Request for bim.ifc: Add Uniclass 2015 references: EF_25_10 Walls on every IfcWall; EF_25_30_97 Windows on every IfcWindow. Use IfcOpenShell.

First a look at what the model holds.

```python
import ifcopenshell

model = ifcopenshell.open("bim.ifc")
print(model.schema)
print("classifications:", [c.Name for c in model.by_type("IfcClassification")])
for ifc_class in ("IfcDoor", "IfcRoof", "IfcStair", "IfcWall", "IfcWindow"):
    print(ifc_class, len(model.by_type(ifc_class)))
```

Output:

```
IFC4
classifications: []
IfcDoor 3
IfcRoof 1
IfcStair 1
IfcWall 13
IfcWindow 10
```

```python
import ifcopenshell
import ifcopenshell.api.classification

model = ifcopenshell.open("bim.ifc")

system = ifcopenshell.api.classification.add_classification(model, classification="Uniclass 2015")

codes = {
    "IfcWall": ("EF_25_10", "Walls"),
    "IfcWindow": ("EF_25_30_97", "Windows"),
}
for ifc_class, (code, name) in codes.items():
    products = model.by_type(ifc_class)
    ifcopenshell.api.classification.add_reference(
        model, products=products, classification=system, identification=code, name=name
    )
    print(code, len(products))

model.write("bim_rev.ifc")
```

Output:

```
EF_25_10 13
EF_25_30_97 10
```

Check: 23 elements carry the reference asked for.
